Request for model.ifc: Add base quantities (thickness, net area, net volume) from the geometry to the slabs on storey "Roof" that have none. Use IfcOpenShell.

First a look at what the model holds.

```python
import ifcopenshell
import ifcopenshell.util.element
import ifcopenshell.util.unit

model = ifcopenshell.open("model.ifc")
print(model.schema)
for unit_type in ("LENGTHUNIT", "AREAUNIT", "VOLUMEUNIT"):
    print(unit_type, ifcopenshell.util.unit.calculate_unit_scale(model, unit_type))
storey = next(s for s in model.by_type("IfcBuildingStorey") if s.Name == "Roof")
slabs = [e for e in ifcopenshell.util.element.get_decomposition(storey) if e.is_a("IfcSlab")]
for e in sorted(slabs, key=lambda e: e.id()):
    print(e.id(), e.is_a(), e.Name, list(ifcopenshell.util.element.get_psets(e, qtos_only=True)), sep=" | ")
```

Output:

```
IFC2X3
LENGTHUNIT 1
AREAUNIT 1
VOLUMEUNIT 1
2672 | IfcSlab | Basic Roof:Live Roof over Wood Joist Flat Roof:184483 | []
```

```python
import ifcopenshell
import ifcopenshell.api.pset
import ifcopenshell.geom
import ifcopenshell.util.element
import ifcopenshell.util.shape
import ifcopenshell.util.unit

model = ifcopenshell.open("model.ifc")
unit_scale = ifcopenshell.util.unit.calculate_unit_scale(model)
area_scale = ifcopenshell.util.unit.calculate_unit_scale(model, "AREAUNIT")
volume_scale = ifcopenshell.util.unit.calculate_unit_scale(model, "VOLUMEUNIT")
settings = ifcopenshell.geom.settings()

storey = next(s for s in model.by_type("IfcBuildingStorey") if s.Name == "Roof")
slabs = [e for e in ifcopenshell.util.element.get_decomposition(storey) if e.is_a("IfcSlab")]

for e in sorted(slabs, key=lambda e: e.id()):
    if ifcopenshell.util.element.get_psets(e, qtos_only=True, should_inherit=False):
        continue
    # Geometry comes back in metres, in the element's own axes.
    shape = ifcopenshell.geom.create_shape(settings, e)
    values = {
        "Width": ifcopenshell.util.shape.get_z(shape.geometry) / unit_scale,
        "NetArea": ifcopenshell.util.shape.get_footprint_area(shape.geometry) / area_scale,
        "NetVolume": ifcopenshell.util.shape.get_volume(shape.geometry) / volume_scale,
    }
    qto = ifcopenshell.api.pset.add_qto(model, product=e, name="BaseQuantities")
    ifcopenshell.api.pset.edit_qto(model, qto=qto, properties=values)
    print(e.id(), {k: round(v, 3) for k, v in values.items()})

model.write("model_edited.ifc")
```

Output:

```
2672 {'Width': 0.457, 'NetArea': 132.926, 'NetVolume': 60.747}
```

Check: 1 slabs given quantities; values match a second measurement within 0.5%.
